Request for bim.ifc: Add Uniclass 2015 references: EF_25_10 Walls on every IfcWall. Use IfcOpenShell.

First a look at what the model holds.

```python
import ifcopenshell

model = ifcopenshell.open("bim.ifc")
print(model.schema)
print("classifications:", [c.Name for c in model.by_type("IfcClassification")])
for ifc_class in ("IfcDoor", "IfcRoof", "IfcStair", "IfcWall", "IfcWindow"):
    print(ifc_class, len(model.by_type(ifc_class)))
```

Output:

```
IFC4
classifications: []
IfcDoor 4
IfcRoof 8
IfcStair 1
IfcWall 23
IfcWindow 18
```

```python
import ifcopenshell
import ifcopenshell.api.classification

model = ifcopenshell.open("bim.ifc")

system = ifcopenshell.api.classification.add_classification(model, classification="Uniclass 2015")

codes = {
    "IfcWall": ("EF_25_10", "Walls"),
}
for ifc_class, (code, name) in codes.items():
    products = model.by_type(ifc_class)
    ifcopenshell.api.classification.add_reference(
        model, products=products, classification=system, identification=code, name=name
    )
    print(code, len(products))

model.write("bim_v2.ifc")
```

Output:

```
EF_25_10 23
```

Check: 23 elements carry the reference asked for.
